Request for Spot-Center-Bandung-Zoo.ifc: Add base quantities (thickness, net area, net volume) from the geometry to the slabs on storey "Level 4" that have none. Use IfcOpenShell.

First a look at what the model holds.

```python
import ifcopenshell
import ifcopenshell.util.element
import ifcopenshell.util.unit

model = ifcopenshell.open("Spot-Center-Bandung-Zoo.ifc")
print(model.schema)
for unit_type in ("LENGTHUNIT", "AREAUNIT", "VOLUMEUNIT"):
    print(unit_type, ifcopenshell.util.unit.calculate_unit_scale(model, unit_type))
storey = next(s for s in model.by_type("IfcBuildingStorey") if s.Name == "Level 4")
slabs = [e for e in ifcopenshell.util.element.get_decomposition(storey) if e.is_a("IfcSlab")]
for e in sorted(slabs, key=lambda e: e.id()):
    print(e.id(), e.is_a(), e.Name, list(ifcopenshell.util.element.get_psets(e, qtos_only=True)), sep=" | ")
```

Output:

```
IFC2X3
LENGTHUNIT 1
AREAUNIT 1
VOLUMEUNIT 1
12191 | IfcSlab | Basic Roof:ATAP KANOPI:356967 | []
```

```python
import ifcopenshell
import ifcopenshell.api.pset
import ifcopenshell.geom
import ifcopenshell.util.element
import ifcopenshell.util.shape
import ifcopenshell.util.unit

model = ifcopenshell.open("Spot-Center-Bandung-Zoo.ifc")
unit_scale = ifcopenshell.util.unit.calculate_unit_scale(model)
area_scale = ifcopenshell.util.unit.calculate_unit_scale(model, "AREAUNIT")
volume_scale = ifcopenshell.util.unit.calculate_unit_scale(model, "VOLUMEUNIT")
settings = ifcopenshell.geom.settings()

storey = next(s for s in model.by_type("IfcBuildingStorey") if s.Name == "Level 4")
slabs = [e for e in ifcopenshell.util.element.get_decomposition(storey) if e.is_a("IfcSlab")]

for e in sorted(slabs, key=lambda e: e.id()):
    if ifcopenshell.util.element.get_psets(e, qtos_only=True, should_inherit=False):
        continue
    # Geometry comes back in metres, in the element's own axes.
    shape = ifcopenshell.geom.create_shape(settings, e)
    values = {
        "Width": ifcopenshell.util.shape.get_z(shape.geometry) / unit_scale,
        "NetArea": ifcopenshell.util.shape.get_footprint_area(shape.geometry) / area_scale,
        "NetVolume": ifcopenshell.util.shape.get_volume(shape.geometry) / volume_scale,
    }
    qto = ifcopenshell.api.pset.add_qto(model, product=e, name="BaseQuantities")
    ifcopenshell.api.pset.edit_qto(model, qto=qto, properties=values)
    print(e.id(), {k: round(v, 3) for k, v in values.items()})

model.write("Spot-Center-Bandung-Zoo_rev.ifc")
```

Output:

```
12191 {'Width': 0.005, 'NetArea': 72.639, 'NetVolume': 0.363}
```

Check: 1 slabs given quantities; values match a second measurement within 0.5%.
